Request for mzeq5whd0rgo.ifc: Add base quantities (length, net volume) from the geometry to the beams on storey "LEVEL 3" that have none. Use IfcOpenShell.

First a look at what the model holds.

```python
import ifcopenshell
import ifcopenshell.util.element
import ifcopenshell.util.unit

model = ifcopenshell.open("mzeq5whd0rgo.ifc")
print(model.schema)
for unit_type in ("LENGTHUNIT", "AREAUNIT", "VOLUMEUNIT"):
    print(unit_type, ifcopenshell.util.unit.calculate_unit_scale(model, unit_type))
storey = next(s for s in model.by_type("IfcBuildingStorey") if s.Name == "LEVEL 3")
beams = [e for e in ifcopenshell.util.element.get_decomposition(storey) if e.is_a("IfcBeam")]
for e in sorted(beams, key=lambda e: e.id()):
    print(e.id(), e.is_a(), e.Name, list(ifcopenshell.util.element.get_psets(e, qtos_only=True)), sep=" | ")
```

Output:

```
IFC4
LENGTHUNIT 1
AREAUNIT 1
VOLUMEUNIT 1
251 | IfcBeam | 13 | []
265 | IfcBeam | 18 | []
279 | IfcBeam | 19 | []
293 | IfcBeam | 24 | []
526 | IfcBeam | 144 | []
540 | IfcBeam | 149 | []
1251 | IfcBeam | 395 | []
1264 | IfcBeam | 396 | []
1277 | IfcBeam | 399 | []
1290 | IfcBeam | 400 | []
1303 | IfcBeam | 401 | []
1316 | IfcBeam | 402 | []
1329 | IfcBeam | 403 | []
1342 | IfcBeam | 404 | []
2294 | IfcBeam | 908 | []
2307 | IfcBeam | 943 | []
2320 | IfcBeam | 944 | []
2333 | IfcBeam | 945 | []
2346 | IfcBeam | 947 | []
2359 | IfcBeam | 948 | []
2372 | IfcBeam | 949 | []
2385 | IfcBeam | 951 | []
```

```python
import ifcopenshell
import ifcopenshell.api.pset
import ifcopenshell.geom
import ifcopenshell.util.element
import ifcopenshell.util.shape
import ifcopenshell.util.unit

model = ifcopenshell.open("mzeq5whd0rgo.ifc")
unit_scale = ifcopenshell.util.unit.calculate_unit_scale(model)
volume_scale = ifcopenshell.util.unit.calculate_unit_scale(model, "VOLUMEUNIT")
settings = ifcopenshell.geom.settings()

storey = next(s for s in model.by_type("IfcBuildingStorey") if s.Name == "LEVEL 3")
beams = [e for e in ifcopenshell.util.element.get_decomposition(storey) if e.is_a("IfcBeam")]

for e in sorted(beams, key=lambda e: e.id()):
    if ifcopenshell.util.element.get_psets(e, qtos_only=True, should_inherit=False):
        continue
    # Geometry comes back in metres, in the element's own axes.
    shape = ifcopenshell.geom.create_shape(settings, e)
    values = {
        "Length": ifcopenshell.util.shape.get_max_xyz(shape.geometry) / unit_scale,
        "NetVolume": ifcopenshell.util.shape.get_volume(shape.geometry) / volume_scale,
    }
    qto = ifcopenshell.api.pset.add_qto(model, product=e, name="Qto_BeamBaseQuantities")
    ifcopenshell.api.pset.edit_qto(model, qto=qto, properties=values)
    print(e.id(), {k: round(v, 3) for k, v in values.items()})

model.write("mzeq5whd0rgo_v2.ifc")
```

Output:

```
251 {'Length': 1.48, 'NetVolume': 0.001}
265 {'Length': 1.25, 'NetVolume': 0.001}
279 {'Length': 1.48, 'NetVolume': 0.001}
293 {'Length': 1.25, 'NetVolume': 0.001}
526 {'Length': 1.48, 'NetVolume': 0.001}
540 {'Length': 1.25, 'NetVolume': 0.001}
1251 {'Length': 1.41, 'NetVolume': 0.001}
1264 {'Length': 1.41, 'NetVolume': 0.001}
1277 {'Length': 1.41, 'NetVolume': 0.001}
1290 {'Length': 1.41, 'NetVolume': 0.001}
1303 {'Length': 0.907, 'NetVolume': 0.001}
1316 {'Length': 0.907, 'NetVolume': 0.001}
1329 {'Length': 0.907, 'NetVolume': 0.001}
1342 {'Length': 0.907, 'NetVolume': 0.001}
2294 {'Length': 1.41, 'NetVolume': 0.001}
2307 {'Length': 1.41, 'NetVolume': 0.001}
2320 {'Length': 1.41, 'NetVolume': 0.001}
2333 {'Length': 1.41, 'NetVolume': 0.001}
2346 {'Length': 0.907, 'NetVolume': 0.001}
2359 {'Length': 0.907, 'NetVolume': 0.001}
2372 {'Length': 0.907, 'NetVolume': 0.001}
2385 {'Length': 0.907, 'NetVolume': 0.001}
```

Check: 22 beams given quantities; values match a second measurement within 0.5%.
